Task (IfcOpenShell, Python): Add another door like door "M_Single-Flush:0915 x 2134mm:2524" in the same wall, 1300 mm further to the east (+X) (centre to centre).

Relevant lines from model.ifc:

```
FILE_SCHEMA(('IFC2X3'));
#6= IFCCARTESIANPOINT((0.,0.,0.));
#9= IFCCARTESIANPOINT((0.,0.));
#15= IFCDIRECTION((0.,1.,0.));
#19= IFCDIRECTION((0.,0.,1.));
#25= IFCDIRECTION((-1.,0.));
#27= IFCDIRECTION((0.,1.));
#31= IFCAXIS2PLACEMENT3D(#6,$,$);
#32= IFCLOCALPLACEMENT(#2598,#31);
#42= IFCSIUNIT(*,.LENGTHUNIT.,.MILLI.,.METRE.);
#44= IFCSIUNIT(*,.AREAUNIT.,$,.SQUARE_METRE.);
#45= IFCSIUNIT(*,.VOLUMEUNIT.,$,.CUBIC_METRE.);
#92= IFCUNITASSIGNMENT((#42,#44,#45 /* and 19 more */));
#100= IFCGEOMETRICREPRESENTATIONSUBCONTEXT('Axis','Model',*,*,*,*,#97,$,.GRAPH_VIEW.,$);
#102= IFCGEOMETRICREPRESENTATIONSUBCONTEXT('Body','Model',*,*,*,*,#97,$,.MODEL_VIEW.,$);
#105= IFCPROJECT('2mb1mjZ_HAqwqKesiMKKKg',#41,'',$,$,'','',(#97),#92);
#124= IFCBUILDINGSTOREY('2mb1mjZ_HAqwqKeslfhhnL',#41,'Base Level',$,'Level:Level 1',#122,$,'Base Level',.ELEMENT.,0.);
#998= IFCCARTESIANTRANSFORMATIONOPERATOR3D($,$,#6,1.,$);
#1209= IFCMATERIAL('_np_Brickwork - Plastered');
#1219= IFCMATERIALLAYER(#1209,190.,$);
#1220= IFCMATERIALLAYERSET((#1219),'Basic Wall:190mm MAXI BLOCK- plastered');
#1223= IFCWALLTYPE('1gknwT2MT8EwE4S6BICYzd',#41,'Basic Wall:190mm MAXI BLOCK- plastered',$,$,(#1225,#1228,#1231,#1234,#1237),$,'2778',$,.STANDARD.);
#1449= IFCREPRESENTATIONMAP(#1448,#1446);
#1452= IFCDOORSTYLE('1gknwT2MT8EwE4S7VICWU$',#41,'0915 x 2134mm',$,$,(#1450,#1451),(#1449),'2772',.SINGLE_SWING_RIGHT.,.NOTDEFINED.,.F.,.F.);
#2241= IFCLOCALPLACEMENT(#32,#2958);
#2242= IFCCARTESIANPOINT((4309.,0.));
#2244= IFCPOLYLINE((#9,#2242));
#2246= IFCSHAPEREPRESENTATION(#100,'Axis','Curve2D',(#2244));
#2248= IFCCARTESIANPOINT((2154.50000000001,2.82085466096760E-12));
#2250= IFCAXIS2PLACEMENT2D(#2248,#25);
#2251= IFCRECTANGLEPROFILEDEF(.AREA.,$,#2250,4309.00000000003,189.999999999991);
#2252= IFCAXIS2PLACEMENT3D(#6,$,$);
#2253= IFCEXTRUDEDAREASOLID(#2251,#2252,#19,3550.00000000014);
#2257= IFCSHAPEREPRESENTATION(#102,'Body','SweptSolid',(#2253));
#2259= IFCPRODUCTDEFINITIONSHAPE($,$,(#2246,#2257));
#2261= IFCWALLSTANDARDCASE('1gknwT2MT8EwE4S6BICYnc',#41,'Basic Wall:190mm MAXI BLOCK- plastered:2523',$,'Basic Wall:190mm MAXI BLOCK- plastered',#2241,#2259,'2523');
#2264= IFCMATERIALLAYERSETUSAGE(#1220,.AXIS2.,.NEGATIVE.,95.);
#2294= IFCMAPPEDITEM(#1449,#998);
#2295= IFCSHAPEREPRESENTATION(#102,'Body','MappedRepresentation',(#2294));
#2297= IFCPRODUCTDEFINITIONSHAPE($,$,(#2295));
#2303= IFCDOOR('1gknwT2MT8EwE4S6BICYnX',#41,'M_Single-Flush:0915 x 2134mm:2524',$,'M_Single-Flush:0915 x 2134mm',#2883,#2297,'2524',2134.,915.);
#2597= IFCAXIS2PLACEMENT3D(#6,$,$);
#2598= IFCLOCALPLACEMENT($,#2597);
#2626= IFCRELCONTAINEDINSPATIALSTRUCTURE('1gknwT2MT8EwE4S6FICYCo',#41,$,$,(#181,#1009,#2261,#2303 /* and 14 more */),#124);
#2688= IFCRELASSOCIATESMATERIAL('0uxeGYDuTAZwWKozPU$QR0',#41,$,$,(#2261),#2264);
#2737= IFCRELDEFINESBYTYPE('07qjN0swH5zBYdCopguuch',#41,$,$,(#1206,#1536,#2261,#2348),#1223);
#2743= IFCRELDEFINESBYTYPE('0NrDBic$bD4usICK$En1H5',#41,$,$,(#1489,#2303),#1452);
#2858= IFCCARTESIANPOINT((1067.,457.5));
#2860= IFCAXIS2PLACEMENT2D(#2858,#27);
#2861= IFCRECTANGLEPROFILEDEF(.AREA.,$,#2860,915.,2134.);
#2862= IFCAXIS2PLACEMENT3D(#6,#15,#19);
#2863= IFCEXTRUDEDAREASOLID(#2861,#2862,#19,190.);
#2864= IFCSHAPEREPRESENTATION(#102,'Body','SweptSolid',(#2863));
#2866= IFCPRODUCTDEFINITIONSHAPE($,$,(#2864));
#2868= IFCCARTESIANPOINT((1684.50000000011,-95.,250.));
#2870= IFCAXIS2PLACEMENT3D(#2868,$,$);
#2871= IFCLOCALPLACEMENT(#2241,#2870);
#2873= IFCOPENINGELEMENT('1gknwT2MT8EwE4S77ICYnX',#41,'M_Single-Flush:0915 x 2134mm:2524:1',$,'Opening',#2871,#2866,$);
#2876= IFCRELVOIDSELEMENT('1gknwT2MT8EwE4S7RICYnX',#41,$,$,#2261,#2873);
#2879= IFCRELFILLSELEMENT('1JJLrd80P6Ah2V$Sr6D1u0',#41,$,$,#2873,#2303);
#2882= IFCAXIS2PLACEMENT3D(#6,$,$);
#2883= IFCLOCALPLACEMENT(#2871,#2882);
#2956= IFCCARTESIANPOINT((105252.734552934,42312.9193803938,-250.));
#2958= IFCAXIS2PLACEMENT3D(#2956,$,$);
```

```python
import ifcopenshell
import ifcopenshell.api.feature
import ifcopenshell.api.geometry
import ifcopenshell.api.root
import ifcopenshell.geom
import ifcopenshell.util.element
import ifcopenshell.util.placement
import ifcopenshell.util.shape
import ifcopenshell.util.unit

model = ifcopenshell.open("model.ifc")
unit_scale = ifcopenshell.util.unit.calculate_unit_scale(model)
settings = ifcopenshell.geom.settings()


def volume(element):
    """Net volume in cubic metres, openings subtracted."""
    shape = ifcopenshell.geom.create_shape(settings, element)
    return ifcopenshell.util.shape.get_volume(shape.geometry)


def reuse_history(source, copy):
    """copy_class also copies each property set's owner history, people and application; keep the originals."""
    for rel in copy.IsDefinedBy:
        if rel.is_a("IfcRelDefinesByProperties") and (history := rel.RelatingPropertyDefinition.OwnerHistory):
            rel.RelatingPropertyDefinition.OwnerHistory = source.OwnerHistory
            ifcopenshell.util.element.remove_deep2(model, history)


door = model.by_guid("1gknwT2MT8EwE4S6BICYnX")
opening = door.FillsVoids[0].RelatingOpeningElement
wall = opening.VoidsElements[0].RelatingBuildingElement
before = volume(wall)
shift = ifcopenshell.util.placement.get_local_placement(wall.ObjectPlacement)[:3, 0] * 1.3 / unit_scale

# copy_class copies the void relationship, type, container and properties, but no geometry.
new_opening = ifcopenshell.api.root.copy_class(model, product=opening)
new_opening.Representation = ifcopenshell.util.element.copy_deep(
    model, opening.Representation, exclude=["IfcGeometricRepresentationContext", "IfcRepresentationMap"]
)
new_opening.Name = "M_Single-Flush:0915 x 2134mm"
new_door = ifcopenshell.api.root.copy_class(model, product=door)
new_door.Representation = ifcopenshell.util.element.copy_deep(
    model, door.Representation, exclude=["IfcGeometricRepresentationContext", "IfcRepresentationMap"]
)
new_door.Name = "M_Single-Flush:0915 x 2134mm"
new_door.Tag = None
reuse_history(door, new_door)
fills = ifcopenshell.api.feature.add_filling(model, opening=new_opening, element=new_door)
fills.OwnerHistory = new_door.OwnerHistory  # required in IFC2X3

for old, new in ((opening, new_opening), (door, new_door)):
    matrix = ifcopenshell.util.placement.get_local_placement(old.ObjectPlacement)
    matrix[:3, 3] += shift
    ifcopenshell.api.geometry.edit_object_placement(model, product=new, matrix=matrix, is_si=False)

after = volume(wall)

print(f"wall volume {before:.3f} -> {after:.3f} m3")

model.write("model_edited.ifc")
```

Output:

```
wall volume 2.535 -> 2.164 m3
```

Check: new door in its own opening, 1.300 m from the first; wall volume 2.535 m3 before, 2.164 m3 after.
